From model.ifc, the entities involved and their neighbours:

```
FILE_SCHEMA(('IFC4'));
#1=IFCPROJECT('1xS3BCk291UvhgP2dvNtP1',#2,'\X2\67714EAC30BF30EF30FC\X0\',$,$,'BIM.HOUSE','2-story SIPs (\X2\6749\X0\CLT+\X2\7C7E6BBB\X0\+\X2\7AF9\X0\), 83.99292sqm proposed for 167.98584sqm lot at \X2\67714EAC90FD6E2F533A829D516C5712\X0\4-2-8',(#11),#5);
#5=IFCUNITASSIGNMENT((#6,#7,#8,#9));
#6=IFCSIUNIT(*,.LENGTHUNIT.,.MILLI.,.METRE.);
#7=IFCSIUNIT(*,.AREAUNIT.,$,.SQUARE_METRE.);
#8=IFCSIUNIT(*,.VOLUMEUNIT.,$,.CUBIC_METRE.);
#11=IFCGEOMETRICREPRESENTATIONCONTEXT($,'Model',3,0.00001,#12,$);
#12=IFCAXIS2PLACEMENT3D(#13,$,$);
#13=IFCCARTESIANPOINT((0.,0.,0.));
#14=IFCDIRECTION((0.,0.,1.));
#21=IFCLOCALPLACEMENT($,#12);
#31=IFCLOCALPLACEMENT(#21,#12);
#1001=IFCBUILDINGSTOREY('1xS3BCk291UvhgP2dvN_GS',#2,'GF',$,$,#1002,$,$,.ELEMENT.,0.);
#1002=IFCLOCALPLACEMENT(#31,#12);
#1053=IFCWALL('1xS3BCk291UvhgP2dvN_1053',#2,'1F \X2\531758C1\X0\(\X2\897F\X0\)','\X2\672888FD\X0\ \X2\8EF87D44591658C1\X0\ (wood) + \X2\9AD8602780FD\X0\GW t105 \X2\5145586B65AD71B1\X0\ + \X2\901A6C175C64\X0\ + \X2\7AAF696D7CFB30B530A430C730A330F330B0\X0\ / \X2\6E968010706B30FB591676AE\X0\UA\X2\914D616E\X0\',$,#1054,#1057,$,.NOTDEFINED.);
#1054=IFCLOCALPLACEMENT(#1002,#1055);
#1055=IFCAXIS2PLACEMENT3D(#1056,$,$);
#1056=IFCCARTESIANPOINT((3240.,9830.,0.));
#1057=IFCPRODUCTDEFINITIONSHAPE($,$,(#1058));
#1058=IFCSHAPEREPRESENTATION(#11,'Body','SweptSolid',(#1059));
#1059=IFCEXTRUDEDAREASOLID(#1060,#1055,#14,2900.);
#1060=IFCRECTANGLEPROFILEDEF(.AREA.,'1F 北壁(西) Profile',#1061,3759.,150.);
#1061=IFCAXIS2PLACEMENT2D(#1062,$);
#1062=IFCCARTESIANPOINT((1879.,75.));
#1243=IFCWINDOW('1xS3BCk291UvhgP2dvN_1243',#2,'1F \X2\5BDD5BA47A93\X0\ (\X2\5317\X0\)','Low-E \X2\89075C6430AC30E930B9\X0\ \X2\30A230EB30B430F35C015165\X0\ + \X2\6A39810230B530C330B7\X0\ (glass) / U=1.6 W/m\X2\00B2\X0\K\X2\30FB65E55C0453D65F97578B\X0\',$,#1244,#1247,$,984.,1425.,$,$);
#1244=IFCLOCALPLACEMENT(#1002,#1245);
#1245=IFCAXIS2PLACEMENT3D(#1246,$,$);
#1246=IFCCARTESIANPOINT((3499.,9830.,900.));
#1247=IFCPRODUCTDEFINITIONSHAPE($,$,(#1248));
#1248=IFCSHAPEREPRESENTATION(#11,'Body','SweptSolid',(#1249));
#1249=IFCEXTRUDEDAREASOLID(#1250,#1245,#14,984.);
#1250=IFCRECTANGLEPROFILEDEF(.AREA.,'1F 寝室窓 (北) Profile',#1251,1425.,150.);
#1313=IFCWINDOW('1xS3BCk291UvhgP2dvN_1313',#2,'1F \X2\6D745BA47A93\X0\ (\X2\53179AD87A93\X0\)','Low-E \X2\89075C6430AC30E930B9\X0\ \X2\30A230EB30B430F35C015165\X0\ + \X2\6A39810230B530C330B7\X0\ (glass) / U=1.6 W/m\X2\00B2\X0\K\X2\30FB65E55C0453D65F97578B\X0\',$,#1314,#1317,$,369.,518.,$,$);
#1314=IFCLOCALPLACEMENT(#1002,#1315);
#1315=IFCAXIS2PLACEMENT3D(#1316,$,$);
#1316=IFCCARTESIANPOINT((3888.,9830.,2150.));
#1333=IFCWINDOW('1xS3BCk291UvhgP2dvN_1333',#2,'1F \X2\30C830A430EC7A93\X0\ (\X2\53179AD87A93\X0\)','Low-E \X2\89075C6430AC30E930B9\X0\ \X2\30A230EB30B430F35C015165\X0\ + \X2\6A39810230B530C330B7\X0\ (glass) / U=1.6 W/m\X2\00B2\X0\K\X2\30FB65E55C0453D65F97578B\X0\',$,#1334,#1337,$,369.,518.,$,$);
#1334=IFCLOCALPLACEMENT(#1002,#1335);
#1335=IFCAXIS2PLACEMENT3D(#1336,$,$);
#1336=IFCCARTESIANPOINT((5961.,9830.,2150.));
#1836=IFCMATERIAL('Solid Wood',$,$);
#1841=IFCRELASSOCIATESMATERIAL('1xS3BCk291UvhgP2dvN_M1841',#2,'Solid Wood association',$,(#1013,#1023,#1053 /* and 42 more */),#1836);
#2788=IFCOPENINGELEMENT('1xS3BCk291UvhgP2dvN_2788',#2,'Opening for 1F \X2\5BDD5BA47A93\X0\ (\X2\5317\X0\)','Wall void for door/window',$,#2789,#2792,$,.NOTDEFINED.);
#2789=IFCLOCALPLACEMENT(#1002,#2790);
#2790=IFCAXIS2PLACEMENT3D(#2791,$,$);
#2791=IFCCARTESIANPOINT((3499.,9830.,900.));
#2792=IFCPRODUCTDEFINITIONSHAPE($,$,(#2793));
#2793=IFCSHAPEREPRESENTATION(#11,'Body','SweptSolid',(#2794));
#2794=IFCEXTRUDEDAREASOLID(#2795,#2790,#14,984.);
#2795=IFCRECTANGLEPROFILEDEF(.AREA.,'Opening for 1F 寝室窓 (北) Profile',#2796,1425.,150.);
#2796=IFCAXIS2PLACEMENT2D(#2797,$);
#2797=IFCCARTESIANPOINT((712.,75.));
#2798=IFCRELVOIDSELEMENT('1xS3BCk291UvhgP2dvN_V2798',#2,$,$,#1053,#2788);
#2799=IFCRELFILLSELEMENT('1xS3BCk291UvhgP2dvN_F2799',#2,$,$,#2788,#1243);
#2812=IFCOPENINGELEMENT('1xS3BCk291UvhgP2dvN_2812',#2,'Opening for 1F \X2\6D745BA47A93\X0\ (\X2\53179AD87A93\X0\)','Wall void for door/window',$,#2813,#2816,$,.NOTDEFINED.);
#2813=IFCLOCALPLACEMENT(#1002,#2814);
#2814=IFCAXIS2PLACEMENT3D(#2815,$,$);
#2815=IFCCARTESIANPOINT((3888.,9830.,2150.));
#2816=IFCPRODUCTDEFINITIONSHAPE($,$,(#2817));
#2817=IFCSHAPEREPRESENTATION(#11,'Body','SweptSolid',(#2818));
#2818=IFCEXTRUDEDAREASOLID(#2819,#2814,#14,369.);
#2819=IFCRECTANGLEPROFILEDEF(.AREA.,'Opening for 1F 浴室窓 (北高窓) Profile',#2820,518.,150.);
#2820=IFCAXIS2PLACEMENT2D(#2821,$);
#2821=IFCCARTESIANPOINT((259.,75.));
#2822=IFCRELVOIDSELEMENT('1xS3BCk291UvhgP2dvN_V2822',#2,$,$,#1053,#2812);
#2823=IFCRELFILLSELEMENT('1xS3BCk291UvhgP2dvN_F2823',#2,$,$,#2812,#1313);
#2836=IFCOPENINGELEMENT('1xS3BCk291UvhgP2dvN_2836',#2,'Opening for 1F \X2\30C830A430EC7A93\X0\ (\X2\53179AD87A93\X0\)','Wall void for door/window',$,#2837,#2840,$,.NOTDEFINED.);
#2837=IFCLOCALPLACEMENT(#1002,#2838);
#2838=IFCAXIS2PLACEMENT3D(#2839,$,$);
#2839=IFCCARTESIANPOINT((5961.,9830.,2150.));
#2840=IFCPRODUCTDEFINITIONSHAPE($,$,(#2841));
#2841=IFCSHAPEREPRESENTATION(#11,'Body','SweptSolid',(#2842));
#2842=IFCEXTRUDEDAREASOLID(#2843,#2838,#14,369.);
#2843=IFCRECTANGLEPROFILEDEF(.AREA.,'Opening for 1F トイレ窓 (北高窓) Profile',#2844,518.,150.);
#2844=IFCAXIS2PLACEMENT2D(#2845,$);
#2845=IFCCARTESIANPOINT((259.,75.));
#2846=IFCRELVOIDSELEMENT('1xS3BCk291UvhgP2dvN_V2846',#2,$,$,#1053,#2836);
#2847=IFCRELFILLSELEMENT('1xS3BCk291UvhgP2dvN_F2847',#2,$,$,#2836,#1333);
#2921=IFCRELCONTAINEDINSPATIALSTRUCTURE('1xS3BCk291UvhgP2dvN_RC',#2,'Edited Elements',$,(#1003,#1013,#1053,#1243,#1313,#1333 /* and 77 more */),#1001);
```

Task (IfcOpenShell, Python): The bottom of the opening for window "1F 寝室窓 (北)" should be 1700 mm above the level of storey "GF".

```python
import numpy as np
import ifcopenshell
import ifcopenshell.api.geometry
import ifcopenshell.geom
import ifcopenshell.util.element
import ifcopenshell.util.placement
import ifcopenshell.util.shape
import ifcopenshell.util.unit

model = ifcopenshell.open("model.ifc")
unit_scale = ifcopenshell.util.unit.calculate_unit_scale(model)

window = model.by_guid("1xS3BCk291UvhgP2dvN_1243")
opening = window.FillsVoids[0].RelatingOpeningElement
storey = ifcopenshell.util.element.get_container(window, ifc_class="IfcBuildingStorey")
level = ifcopenshell.util.placement.get_local_placement(storey.ObjectPlacement)[2, 3]

# The opening's origin need not be at the sill, so measure its lowest point.
shape = ifcopenshell.geom.create_shape(ifcopenshell.geom.settings(), opening)
bottom = ifcopenshell.util.shape.get_shape_bottom_elevation(shape, shape.geometry) / unit_scale
dz = level + 1.7 / unit_scale - bottom

shift = np.array([0.0, 0.0, dz])
# The window is not placed relative to its opening, so move both.
for product in (opening, window):
    matrix = ifcopenshell.util.placement.get_local_placement(product.ObjectPlacement)
    matrix[:3, 3] += shift
    ifcopenshell.api.geometry.edit_object_placement(model, product=product, matrix=matrix, is_si=False)

print(f"moved by {dz * unit_scale:+.3f} m")

model.write("model_v2.ifc")
```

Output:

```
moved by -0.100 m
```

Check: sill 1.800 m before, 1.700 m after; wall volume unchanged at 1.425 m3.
